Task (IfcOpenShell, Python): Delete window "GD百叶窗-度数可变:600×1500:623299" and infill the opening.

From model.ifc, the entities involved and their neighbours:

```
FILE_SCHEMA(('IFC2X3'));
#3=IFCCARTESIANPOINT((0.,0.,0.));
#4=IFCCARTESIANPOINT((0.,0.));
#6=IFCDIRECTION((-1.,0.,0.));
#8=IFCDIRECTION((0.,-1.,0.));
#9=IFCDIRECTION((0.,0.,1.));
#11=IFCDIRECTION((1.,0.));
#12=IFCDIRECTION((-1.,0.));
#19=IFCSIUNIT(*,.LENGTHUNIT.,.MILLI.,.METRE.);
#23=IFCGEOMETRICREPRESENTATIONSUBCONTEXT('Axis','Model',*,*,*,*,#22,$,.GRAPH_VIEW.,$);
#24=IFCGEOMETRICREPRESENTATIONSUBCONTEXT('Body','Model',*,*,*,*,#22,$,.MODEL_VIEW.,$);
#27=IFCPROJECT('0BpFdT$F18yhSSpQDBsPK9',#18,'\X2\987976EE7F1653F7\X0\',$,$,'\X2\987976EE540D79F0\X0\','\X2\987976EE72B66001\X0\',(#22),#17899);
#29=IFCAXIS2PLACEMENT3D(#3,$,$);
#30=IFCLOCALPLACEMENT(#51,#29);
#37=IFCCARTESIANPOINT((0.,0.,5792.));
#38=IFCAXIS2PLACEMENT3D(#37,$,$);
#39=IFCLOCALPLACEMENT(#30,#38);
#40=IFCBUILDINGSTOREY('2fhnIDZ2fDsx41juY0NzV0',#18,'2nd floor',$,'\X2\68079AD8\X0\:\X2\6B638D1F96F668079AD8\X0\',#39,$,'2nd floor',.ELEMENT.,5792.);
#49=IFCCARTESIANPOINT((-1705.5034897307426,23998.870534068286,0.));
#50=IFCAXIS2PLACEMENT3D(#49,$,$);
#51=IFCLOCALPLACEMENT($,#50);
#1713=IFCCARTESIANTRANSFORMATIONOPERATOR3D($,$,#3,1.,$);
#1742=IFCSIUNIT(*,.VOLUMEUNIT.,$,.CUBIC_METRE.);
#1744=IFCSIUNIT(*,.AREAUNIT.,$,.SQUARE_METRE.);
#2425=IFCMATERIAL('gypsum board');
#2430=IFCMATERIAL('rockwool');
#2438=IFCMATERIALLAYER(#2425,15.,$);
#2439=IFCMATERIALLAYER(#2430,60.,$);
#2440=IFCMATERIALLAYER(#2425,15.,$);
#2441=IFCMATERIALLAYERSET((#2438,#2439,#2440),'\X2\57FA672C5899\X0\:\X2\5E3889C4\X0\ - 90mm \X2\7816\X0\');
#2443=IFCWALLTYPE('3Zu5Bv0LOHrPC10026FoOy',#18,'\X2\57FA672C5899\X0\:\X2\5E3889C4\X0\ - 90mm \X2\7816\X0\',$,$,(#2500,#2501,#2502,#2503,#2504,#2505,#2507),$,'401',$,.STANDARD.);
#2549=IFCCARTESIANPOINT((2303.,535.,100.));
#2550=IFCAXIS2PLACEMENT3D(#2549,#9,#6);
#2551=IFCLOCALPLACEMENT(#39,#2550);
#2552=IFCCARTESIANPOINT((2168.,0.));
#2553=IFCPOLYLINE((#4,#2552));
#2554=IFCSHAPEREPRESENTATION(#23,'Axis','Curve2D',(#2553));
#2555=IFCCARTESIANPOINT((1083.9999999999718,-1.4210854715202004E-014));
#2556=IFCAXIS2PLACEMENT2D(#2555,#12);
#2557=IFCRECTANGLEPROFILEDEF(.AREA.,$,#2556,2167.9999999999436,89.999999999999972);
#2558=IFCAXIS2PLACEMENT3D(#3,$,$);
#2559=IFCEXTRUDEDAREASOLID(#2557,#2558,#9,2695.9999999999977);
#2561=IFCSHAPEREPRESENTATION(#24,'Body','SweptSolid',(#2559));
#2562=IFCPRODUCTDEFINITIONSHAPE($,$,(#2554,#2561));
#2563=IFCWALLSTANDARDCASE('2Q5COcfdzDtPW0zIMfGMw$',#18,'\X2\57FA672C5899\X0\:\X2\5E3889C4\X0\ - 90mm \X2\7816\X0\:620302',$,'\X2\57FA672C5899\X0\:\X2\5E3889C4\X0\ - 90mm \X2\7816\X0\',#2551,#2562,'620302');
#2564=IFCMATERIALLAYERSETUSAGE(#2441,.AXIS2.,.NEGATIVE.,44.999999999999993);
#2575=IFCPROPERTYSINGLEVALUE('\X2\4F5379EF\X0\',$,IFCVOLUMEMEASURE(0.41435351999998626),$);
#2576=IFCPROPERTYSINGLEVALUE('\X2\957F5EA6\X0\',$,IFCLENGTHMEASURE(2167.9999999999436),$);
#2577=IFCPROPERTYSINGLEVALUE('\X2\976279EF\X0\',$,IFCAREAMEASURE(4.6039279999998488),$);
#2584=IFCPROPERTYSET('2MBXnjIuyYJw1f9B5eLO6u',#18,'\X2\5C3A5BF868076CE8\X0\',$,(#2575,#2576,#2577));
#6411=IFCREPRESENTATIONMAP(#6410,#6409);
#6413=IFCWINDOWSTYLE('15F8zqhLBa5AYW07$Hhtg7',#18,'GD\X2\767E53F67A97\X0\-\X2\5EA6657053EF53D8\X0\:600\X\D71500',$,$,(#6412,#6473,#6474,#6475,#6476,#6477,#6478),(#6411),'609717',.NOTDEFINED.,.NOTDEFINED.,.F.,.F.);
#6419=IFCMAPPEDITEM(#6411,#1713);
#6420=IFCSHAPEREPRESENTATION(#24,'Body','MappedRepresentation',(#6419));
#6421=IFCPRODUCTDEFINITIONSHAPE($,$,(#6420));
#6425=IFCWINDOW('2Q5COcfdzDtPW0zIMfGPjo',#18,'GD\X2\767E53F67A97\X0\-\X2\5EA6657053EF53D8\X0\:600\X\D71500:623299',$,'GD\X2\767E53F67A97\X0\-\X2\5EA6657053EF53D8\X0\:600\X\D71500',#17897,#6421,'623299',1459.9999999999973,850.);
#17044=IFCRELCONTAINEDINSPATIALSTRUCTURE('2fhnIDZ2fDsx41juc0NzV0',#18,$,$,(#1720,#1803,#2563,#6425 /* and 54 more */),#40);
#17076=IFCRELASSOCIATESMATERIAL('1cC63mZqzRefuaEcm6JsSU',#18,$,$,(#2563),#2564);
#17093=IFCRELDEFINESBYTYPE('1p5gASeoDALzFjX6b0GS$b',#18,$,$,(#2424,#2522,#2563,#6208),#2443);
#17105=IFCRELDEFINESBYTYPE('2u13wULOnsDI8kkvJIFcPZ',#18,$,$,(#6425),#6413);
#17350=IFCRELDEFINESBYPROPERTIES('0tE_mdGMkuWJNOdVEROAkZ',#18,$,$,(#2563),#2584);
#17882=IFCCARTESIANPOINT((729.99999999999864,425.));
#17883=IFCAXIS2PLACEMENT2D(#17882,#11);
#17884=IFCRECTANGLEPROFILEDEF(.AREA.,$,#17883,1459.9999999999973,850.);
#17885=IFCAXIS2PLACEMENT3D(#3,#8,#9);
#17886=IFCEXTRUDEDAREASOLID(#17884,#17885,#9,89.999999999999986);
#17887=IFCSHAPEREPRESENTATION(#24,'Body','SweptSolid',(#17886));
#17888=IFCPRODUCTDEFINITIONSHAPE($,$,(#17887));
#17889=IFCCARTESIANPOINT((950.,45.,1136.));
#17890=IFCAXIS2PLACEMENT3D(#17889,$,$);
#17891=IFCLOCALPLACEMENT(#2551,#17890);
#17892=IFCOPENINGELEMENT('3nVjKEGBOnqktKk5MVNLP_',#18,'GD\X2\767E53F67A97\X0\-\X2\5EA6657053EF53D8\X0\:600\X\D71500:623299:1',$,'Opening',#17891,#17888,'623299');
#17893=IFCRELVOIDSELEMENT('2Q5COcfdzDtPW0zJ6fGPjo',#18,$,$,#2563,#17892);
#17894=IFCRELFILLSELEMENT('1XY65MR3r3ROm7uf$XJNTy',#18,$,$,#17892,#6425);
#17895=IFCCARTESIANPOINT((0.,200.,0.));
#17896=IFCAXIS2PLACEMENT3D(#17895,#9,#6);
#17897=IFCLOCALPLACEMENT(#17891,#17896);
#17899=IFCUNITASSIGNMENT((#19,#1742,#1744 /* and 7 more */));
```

```python
import ifcopenshell
import ifcopenshell.api.feature
import ifcopenshell.api.pset
import ifcopenshell.api.root
import ifcopenshell.geom
import ifcopenshell.util.element
import ifcopenshell.util.shape
import ifcopenshell.util.unit

model = ifcopenshell.open("model.ifc")
area_scale = ifcopenshell.util.unit.calculate_unit_scale(model, "AREAUNIT")
volume_scale = ifcopenshell.util.unit.calculate_unit_scale(model, "VOLUMEUNIT")
settings = ifcopenshell.geom.settings()


def volume(element):
    """Net volume in cubic metres, openings subtracted."""
    shape = ifcopenshell.geom.create_shape(settings, element)
    return ifcopenshell.util.shape.get_volume(shape.geometry)


window = model.by_guid("2Q5COcfdzDtPW0zIMfGPjo")
opening = window.FillsVoids[0].RelatingOpeningElement
wall = opening.VoidsElements[0].RelatingBuildingElement
before = volume(wall)

ifcopenshell.api.root.remove_product(model, product=window)
ifcopenshell.api.feature.remove_feature(model, feature=opening)

after = volume(wall)
thickness = 0.09  # wall thickness in metres

# Update the wall's stored quantities.
pset = model.by_id(ifcopenshell.util.element.get_pset(wall, "尺寸标注", should_inherit=False)["id"])
ifcopenshell.api.pset.edit_pset(model, pset=pset, properties={
    "体积": model.create_entity("IfcVolumeMeasure", after / volume_scale),
    "面积": model.create_entity("IfcAreaMeasure", after / thickness / area_scale),
})

print(f"wall volume {before:.3f} -> {after:.3f} m3")

model.write("model_edited.ifc")
```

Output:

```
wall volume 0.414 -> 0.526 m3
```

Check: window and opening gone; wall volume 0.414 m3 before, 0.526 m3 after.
